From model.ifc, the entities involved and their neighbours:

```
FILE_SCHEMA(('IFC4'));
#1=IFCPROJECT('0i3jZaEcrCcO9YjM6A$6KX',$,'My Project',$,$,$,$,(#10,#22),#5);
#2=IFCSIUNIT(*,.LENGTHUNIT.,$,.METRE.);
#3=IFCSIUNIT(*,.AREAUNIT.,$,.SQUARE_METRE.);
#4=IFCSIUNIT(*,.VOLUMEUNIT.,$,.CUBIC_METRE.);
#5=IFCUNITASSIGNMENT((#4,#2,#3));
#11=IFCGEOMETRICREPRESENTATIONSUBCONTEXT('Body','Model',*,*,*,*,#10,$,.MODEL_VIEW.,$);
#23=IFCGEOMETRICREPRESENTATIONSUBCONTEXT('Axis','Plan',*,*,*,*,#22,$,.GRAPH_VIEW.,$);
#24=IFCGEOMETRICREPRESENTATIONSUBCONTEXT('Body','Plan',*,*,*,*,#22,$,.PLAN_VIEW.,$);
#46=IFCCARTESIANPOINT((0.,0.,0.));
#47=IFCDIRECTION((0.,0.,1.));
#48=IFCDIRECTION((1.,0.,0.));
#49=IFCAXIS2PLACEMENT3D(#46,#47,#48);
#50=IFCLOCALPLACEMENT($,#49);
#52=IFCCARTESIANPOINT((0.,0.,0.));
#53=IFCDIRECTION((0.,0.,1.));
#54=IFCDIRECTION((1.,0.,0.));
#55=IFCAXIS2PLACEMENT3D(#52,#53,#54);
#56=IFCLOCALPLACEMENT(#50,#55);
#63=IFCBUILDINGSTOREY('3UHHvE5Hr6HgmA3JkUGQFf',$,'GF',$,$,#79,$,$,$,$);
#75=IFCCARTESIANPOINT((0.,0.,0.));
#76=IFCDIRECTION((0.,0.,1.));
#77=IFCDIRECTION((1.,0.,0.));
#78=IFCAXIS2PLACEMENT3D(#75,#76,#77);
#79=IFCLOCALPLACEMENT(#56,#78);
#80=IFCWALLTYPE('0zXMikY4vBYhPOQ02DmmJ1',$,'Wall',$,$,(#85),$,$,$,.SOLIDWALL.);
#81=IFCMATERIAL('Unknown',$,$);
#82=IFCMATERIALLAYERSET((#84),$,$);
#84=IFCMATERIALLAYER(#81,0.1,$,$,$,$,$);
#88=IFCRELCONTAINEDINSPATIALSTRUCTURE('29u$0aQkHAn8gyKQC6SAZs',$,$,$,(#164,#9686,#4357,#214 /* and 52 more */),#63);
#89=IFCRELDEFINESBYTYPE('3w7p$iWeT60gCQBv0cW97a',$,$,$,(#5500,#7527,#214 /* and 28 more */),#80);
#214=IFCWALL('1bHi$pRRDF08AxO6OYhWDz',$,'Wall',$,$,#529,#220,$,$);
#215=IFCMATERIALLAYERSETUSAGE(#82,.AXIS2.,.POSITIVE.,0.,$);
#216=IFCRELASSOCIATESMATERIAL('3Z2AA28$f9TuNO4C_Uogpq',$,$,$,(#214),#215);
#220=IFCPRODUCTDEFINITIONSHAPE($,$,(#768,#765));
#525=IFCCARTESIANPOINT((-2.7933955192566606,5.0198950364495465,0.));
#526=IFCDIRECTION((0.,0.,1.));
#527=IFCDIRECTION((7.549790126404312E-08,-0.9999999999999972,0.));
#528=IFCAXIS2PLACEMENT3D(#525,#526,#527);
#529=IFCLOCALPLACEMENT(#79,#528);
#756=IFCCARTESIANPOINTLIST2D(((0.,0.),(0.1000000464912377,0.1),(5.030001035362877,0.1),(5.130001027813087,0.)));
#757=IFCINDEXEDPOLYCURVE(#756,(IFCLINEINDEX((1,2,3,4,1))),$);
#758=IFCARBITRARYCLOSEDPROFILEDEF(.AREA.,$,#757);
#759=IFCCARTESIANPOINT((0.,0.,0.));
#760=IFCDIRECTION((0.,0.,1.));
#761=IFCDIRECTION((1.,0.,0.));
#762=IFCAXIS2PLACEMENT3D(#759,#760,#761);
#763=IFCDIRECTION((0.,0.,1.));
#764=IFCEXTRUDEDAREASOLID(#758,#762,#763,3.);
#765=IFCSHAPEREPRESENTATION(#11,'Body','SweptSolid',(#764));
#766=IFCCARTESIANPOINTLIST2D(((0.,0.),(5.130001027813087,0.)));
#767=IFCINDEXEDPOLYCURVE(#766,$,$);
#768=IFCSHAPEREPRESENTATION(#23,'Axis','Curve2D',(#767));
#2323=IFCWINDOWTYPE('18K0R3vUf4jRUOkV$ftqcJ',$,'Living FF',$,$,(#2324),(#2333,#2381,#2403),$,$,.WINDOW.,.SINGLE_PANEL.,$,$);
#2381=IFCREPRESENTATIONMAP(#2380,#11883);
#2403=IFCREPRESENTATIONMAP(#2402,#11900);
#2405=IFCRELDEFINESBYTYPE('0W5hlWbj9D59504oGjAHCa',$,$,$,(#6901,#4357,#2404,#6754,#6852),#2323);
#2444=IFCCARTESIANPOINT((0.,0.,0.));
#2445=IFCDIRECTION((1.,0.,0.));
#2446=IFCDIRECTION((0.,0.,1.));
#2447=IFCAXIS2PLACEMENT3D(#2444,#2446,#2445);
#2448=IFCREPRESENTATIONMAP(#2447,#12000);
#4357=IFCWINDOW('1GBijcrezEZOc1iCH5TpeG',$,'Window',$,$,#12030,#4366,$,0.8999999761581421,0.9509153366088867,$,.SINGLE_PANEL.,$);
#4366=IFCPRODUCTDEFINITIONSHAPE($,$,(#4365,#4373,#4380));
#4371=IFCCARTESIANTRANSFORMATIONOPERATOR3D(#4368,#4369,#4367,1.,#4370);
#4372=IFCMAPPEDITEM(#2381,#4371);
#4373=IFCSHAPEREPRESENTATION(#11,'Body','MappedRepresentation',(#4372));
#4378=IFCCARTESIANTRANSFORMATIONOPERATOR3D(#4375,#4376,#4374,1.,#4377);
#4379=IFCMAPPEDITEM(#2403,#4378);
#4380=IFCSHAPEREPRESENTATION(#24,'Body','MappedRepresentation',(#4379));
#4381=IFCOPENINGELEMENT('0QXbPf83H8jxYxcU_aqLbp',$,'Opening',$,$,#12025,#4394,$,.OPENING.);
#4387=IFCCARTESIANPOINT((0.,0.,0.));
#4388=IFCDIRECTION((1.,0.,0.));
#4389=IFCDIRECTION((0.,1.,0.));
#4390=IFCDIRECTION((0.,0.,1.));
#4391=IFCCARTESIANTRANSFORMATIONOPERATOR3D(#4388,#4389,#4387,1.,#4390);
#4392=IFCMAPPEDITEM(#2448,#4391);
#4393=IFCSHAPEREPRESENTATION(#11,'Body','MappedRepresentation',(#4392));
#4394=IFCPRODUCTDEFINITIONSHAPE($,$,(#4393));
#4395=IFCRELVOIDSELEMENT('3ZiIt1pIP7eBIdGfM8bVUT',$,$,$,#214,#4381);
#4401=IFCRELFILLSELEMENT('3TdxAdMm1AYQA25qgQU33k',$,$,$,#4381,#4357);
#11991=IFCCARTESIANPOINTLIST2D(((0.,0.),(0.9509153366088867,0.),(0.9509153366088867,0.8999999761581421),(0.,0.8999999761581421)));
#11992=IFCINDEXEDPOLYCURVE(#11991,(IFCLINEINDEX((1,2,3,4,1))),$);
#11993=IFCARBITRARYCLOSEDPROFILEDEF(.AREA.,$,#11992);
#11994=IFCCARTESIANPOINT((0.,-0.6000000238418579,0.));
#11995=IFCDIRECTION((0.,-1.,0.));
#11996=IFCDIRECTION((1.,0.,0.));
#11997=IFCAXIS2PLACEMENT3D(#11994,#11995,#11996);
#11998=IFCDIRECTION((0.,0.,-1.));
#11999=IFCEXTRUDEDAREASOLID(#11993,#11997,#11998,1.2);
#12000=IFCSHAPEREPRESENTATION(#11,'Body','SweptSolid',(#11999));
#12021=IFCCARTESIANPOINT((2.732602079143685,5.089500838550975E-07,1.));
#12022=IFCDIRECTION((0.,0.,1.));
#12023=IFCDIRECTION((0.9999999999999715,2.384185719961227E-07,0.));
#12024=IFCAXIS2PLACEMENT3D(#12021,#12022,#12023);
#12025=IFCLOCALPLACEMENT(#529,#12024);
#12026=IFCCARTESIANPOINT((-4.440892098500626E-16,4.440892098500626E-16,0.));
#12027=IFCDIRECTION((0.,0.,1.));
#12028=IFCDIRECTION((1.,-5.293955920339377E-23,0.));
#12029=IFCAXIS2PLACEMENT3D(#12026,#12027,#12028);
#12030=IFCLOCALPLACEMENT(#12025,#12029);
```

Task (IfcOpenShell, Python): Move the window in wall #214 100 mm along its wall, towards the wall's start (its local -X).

```python
import ifcopenshell
import ifcopenshell.api.geometry
import ifcopenshell.util.placement

model = ifcopenshell.open("model.ifc")

window = model.by_guid("1GBijcrezEZOc1iCH5TpeG")
opening = window.FillsVoids[0].RelatingOpeningElement
wall = opening.VoidsElements[0].RelatingBuildingElement

wall_matrix = ifcopenshell.util.placement.get_local_placement(wall.ObjectPlacement)
shift = wall_matrix[:3, 0] * -0.1
before = ifcopenshell.util.placement.get_local_placement(window.ObjectPlacement)[:3, 3].copy()

# The window is placed relative to its opening, so it follows when the opening moves.
matrix = ifcopenshell.util.placement.get_local_placement(opening.ObjectPlacement)
matrix[:3, 3] += shift
ifcopenshell.api.geometry.edit_object_placement(
    model, product=opening, matrix=matrix, is_si=False, should_transform_children=True
)

after = ifcopenshell.util.placement.get_local_placement(window.ObjectPlacement)[:3, 3]
print("window moved by", (after - before).round(3) + 0.0)

model.write("model_edited.ifc")
```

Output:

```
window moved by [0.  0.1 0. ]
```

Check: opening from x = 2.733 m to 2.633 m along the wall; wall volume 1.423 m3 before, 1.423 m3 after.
